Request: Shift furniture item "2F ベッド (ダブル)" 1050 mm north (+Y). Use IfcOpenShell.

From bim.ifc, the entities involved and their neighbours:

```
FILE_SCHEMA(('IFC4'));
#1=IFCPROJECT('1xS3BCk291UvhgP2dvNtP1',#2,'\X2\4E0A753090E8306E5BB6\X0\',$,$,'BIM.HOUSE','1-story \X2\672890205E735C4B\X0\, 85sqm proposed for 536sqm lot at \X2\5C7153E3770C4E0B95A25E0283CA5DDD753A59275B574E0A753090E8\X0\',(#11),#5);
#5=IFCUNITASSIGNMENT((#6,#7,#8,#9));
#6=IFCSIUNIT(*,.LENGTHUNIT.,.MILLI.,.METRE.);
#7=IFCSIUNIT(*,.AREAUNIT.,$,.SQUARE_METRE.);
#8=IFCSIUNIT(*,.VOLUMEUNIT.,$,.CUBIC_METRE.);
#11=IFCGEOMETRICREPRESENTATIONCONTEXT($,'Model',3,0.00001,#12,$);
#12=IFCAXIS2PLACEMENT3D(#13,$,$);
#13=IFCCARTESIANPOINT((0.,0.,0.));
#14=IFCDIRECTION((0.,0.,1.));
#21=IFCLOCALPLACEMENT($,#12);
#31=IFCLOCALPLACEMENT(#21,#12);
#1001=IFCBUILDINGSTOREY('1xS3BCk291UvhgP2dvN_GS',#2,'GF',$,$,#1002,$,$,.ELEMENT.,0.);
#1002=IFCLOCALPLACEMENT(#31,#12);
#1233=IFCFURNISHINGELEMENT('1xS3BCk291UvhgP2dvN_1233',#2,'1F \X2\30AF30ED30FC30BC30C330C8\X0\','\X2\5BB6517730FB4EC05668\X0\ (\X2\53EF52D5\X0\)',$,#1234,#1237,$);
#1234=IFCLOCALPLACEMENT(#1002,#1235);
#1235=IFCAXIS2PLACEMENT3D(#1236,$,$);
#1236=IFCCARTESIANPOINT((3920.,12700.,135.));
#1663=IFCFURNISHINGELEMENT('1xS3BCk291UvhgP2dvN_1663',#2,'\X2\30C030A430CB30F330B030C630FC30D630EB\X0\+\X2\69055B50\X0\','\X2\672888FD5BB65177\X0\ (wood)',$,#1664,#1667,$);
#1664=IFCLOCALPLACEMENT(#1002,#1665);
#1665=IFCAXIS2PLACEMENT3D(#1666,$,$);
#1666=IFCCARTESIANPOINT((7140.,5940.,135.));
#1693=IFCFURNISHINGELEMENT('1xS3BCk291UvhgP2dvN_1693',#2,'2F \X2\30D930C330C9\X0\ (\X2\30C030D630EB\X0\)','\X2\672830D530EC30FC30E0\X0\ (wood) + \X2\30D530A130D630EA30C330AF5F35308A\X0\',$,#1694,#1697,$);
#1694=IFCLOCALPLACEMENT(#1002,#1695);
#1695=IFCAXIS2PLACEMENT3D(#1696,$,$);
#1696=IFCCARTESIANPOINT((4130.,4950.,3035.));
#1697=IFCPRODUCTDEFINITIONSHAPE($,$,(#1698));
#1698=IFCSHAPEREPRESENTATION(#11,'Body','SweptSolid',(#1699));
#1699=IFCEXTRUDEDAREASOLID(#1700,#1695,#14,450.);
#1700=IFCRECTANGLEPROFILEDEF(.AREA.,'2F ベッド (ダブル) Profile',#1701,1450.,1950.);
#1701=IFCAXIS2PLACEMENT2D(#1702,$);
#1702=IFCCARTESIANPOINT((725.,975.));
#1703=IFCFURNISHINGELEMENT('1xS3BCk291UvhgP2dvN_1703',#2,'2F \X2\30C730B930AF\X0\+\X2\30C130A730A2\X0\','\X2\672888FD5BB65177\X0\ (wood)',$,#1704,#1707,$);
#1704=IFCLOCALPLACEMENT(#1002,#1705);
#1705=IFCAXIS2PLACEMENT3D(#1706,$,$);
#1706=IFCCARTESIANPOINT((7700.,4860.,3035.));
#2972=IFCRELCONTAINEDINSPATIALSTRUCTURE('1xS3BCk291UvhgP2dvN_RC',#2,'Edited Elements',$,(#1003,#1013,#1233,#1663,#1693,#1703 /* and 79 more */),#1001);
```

```python
import ifcopenshell
import ifcopenshell.api.geometry
import ifcopenshell.util.placement
import ifcopenshell.util.unit

model = ifcopenshell.open("bim.ifc")
unit_scale = ifcopenshell.util.unit.calculate_unit_scale(model)

item = model.by_guid("1xS3BCk291UvhgP2dvN_1693")
matrix = ifcopenshell.util.placement.get_local_placement(item.ObjectPlacement)
matrix[1, 3] += 1.05 / unit_scale
ifcopenshell.api.geometry.edit_object_placement(model, product=item, matrix=matrix, is_si=False)

print(ifcopenshell.util.placement.get_local_placement(item.ObjectPlacement).round(3) + 0.0)

model.write("bim_v2.ifc")
```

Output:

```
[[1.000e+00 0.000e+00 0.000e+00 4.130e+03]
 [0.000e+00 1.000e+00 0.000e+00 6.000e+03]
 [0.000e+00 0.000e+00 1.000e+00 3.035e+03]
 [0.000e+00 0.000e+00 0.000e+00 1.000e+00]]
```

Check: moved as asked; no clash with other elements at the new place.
